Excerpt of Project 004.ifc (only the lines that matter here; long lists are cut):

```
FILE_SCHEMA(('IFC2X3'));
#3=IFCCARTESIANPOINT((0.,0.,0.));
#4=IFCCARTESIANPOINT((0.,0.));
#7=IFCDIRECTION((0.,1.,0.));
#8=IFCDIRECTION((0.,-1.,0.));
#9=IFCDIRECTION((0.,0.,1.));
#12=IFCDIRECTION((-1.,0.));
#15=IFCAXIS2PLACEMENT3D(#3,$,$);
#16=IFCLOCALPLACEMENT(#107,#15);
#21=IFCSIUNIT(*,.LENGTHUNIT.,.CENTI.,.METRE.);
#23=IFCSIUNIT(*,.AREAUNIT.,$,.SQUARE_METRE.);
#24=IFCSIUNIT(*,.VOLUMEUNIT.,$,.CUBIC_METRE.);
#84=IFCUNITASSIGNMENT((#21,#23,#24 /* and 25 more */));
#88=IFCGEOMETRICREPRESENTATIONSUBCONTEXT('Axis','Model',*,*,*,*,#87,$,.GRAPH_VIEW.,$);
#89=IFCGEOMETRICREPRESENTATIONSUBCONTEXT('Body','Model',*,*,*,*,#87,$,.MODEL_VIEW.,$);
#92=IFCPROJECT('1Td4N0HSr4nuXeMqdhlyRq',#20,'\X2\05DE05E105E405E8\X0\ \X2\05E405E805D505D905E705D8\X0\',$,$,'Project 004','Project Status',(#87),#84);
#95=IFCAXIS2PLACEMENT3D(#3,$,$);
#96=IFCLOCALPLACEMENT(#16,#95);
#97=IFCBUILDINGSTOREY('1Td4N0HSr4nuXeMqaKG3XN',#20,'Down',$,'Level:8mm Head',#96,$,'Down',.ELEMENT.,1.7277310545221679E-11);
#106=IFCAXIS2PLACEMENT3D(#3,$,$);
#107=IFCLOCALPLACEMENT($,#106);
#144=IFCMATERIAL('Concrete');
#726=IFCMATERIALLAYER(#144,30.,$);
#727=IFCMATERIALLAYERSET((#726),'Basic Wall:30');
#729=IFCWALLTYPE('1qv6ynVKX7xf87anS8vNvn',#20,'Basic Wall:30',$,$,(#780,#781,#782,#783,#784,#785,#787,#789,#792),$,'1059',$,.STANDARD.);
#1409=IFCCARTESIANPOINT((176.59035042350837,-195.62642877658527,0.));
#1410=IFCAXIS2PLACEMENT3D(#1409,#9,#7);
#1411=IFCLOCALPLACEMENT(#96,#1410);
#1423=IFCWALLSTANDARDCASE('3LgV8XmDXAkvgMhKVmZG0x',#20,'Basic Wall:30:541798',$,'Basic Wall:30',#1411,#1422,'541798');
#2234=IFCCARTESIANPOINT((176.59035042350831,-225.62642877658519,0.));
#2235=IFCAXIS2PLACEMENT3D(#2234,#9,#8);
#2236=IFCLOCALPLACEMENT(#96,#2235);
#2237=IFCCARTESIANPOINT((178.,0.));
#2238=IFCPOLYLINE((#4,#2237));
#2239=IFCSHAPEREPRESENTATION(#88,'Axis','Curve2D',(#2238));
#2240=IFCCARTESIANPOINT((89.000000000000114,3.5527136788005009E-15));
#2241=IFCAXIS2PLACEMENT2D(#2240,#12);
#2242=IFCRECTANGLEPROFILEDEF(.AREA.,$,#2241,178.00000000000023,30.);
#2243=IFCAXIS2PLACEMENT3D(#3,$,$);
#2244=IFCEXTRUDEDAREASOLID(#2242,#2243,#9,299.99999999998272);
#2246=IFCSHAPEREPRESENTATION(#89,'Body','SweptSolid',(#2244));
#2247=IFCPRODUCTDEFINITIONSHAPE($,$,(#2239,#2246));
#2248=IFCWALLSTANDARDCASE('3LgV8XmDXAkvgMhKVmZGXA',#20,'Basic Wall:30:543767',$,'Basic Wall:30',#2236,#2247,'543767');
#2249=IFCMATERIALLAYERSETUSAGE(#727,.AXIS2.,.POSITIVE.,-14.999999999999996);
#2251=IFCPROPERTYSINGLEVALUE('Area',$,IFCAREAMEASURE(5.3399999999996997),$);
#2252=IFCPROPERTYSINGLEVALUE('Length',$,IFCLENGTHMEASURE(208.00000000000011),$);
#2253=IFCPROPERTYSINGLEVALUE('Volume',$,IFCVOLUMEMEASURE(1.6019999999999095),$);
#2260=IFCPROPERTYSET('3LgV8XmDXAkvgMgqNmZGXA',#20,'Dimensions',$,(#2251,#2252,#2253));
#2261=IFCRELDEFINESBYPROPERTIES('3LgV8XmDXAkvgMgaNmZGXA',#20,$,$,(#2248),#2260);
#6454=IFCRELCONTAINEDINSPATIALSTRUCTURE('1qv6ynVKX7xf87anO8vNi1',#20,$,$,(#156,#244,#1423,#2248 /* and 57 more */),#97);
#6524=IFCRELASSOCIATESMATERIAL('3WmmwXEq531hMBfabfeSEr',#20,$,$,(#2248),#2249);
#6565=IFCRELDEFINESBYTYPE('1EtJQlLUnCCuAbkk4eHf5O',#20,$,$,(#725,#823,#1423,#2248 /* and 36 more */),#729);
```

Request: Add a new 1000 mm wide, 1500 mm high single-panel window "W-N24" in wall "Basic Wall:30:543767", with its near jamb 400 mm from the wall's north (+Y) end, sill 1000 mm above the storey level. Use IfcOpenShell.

```python
import numpy as np
import ifcopenshell
import ifcopenshell.api.feature
import ifcopenshell.api.geometry
import ifcopenshell.api.pset
import ifcopenshell.api.root
import ifcopenshell.api.spatial
import ifcopenshell.api.type
import ifcopenshell.geom
import ifcopenshell.util.element
import ifcopenshell.util.placement
import ifcopenshell.util.representation
import ifcopenshell.util.shape
import ifcopenshell.util.unit

model = ifcopenshell.open("Project 004.ifc")
unit_scale = ifcopenshell.util.unit.calculate_unit_scale(model)
area_scale = ifcopenshell.util.unit.calculate_unit_scale(model, "AREAUNIT")
volume_scale = ifcopenshell.util.unit.calculate_unit_scale(model, "VOLUMEUNIT")
settings = ifcopenshell.geom.settings()


def volume(element):
    """Net volume in cubic metres, openings subtracted."""
    shape = ifcopenshell.geom.create_shape(settings, element)
    return ifcopenshell.util.shape.get_volume(shape.geometry)


wall = model.by_guid("3LgV8XmDXAkvgMhKVmZGXA")
storey = ifcopenshell.util.element.get_container(wall, ifc_class="IfcBuildingStorey")
context = ifcopenshell.util.representation.get_context(model, "Model", "Body", "MODEL_VIEW")
before = volume(wall)

width, height, from_end, sill = 1, 1.5, 0.4, 1  # metres

# The wall runs along its own X axis, and the end named is its -X end.
wall_shape = ifcopenshell.geom.create_shape(settings, wall)
x, y, z = ifcopenshell.util.shape.get_vertices(wall_shape.geometry).T
start = x.min() + from_end
face, thickness = float(y.min()), float(y.max() - y.min())
wall_matrix = ifcopenshell.util.placement.get_local_placement(wall.ObjectPlacement)
level = ifcopenshell.util.placement.get_local_placement(storey.ObjectPlacement)[2, 3]


def in_wall(x, y):
    """Placement at x, y metres in the wall's axes, at sill height."""
    matrix = wall_matrix.copy()
    matrix[:, 3] = wall_matrix @ np.array([x / unit_scale, y / unit_scale, 0.0, 1.0])
    matrix[2, 3] = level + sill / unit_scale
    return matrix


# Opening: a box that overshoots both wall faces by 50 mm.
opening = ifcopenshell.api.root.create_entity(model, ifc_class="IfcOpeningElement")
box = ifcopenshell.api.geometry.add_wall_representation(
    model, context=context, length=width, height=height, thickness=thickness + 0.1
)
ifcopenshell.api.geometry.assign_representation(model, product=opening, representation=box)
ifcopenshell.api.geometry.edit_object_placement(model, product=opening, matrix=in_wall(start, face - 0.05), is_si=False)
ifcopenshell.api.feature.add_feature(model, feature=opening, element=wall)

window = ifcopenshell.api.root.create_entity(model, ifc_class="IfcWindow", name="W-N24")
window.OverallWidth, window.OverallHeight = width / unit_scale, height / unit_scale
body = ifcopenshell.api.geometry.add_window_representation(
    model,
    context=context,
    overall_width=window.OverallWidth,
    overall_height=window.OverallHeight,
    partition_type="SINGLE_PANEL",
)
ifcopenshell.api.geometry.assign_representation(model, product=window, representation=body)
ifcopenshell.api.spatial.assign_container(model, products=[window], relating_structure=storey)
fills = ifcopenshell.api.feature.add_filling(model, opening=opening, element=window)
fills.OwnerHistory = window.OwnerHistory  # required in IFC2X3

# IFC2X3 keeps the operation on the window style.
style = ifcopenshell.api.root.create_entity(model, ifc_class="IfcWindowStyle", name="W-N24")
style.OperationType, style.ConstructionType = "SINGLE_PANEL", "NOTDEFINED"
style.ParameterTakesPrecedence = style.Sizeable = False
ifcopenshell.api.type.assign_type(model, related_objects=[window], relating_type=style)

# Centre the window in the wall's thickness.
ifcopenshell.api.geometry.edit_object_placement(model, product=window, matrix=in_wall(start, face), is_si=False)
window_shape = ifcopenshell.geom.create_shape(settings, window)
depth = ifcopenshell.util.shape.get_vertices(window_shape.geometry)[:, 1]
offset = face + thickness / 2 - (depth.min() + depth.max()) / 2
ifcopenshell.api.geometry.edit_object_placement(model, product=window, matrix=in_wall(start, offset), is_si=False)

after = volume(wall)

# Update the wall's stored quantities.
pset = model.by_id(ifcopenshell.util.element.get_pset(wall, "Dimensions", should_inherit=False)["id"])
ifcopenshell.api.pset.edit_pset(model, pset=pset, properties={
    "Area": model.create_entity("IfcAreaMeasure", after / thickness / area_scale),
    "Volume": model.create_entity("IfcVolumeMeasure", after / volume_scale),
})

print(f"wall volume {before:.3f} -> {after:.3f} m3")

model.write("Project 004_rev.ifc")
```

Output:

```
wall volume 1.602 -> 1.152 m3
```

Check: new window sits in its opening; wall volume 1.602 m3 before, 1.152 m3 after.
